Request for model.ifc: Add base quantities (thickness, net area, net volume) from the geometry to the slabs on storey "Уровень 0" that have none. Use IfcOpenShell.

First a look at what the model holds.

```python
import ifcopenshell
import ifcopenshell.util.element
import ifcopenshell.util.unit

model = ifcopenshell.open("model.ifc")
print(model.schema)
for unit_type in ("LENGTHUNIT", "AREAUNIT", "VOLUMEUNIT"):
    print(unit_type, ifcopenshell.util.unit.calculate_unit_scale(model, unit_type))
storey = next(s for s in model.by_type("IfcBuildingStorey") if s.Name == "Уровень 0")
slabs = [e for e in ifcopenshell.util.element.get_decomposition(storey) if e.is_a("IfcSlab")]
for e in sorted(slabs, key=lambda e: e.id()):
    print(e.id(), e.is_a(), e.Name, list(ifcopenshell.util.element.get_psets(e, qtos_only=True)), sep=" | ")
```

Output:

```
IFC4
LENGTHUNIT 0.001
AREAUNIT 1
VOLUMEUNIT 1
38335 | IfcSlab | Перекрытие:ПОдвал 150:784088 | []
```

```python
import ifcopenshell
import ifcopenshell.api.pset
import ifcopenshell.geom
import ifcopenshell.util.element
import ifcopenshell.util.shape
import ifcopenshell.util.unit

model = ifcopenshell.open("model.ifc")
unit_scale = ifcopenshell.util.unit.calculate_unit_scale(model)
area_scale = ifcopenshell.util.unit.calculate_unit_scale(model, "AREAUNIT")
volume_scale = ifcopenshell.util.unit.calculate_unit_scale(model, "VOLUMEUNIT")
settings = ifcopenshell.geom.settings()

storey = next(s for s in model.by_type("IfcBuildingStorey") if s.Name == "Уровень 0")
slabs = [e for e in ifcopenshell.util.element.get_decomposition(storey) if e.is_a("IfcSlab")]

for e in sorted(slabs, key=lambda e: e.id()):
    if ifcopenshell.util.element.get_psets(e, qtos_only=True, should_inherit=False):
        continue
    # Geometry comes back in metres, in the element's own axes.
    shape = ifcopenshell.geom.create_shape(settings, e)
    values = {
        "Width": ifcopenshell.util.shape.get_z(shape.geometry) / unit_scale,
        "NetArea": ifcopenshell.util.shape.get_footprint_area(shape.geometry) / area_scale,
        "NetVolume": ifcopenshell.util.shape.get_volume(shape.geometry) / volume_scale,
    }
    qto = ifcopenshell.api.pset.add_qto(model, product=e, name="Qto_SlabBaseQuantities")
    ifcopenshell.api.pset.edit_qto(model, qto=qto, properties=values)
    print(e.id(), {k: round(v, 3) for k, v in values.items()})

model.write("model_v2.ifc")
```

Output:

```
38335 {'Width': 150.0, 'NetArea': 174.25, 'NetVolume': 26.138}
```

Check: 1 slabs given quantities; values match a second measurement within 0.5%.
